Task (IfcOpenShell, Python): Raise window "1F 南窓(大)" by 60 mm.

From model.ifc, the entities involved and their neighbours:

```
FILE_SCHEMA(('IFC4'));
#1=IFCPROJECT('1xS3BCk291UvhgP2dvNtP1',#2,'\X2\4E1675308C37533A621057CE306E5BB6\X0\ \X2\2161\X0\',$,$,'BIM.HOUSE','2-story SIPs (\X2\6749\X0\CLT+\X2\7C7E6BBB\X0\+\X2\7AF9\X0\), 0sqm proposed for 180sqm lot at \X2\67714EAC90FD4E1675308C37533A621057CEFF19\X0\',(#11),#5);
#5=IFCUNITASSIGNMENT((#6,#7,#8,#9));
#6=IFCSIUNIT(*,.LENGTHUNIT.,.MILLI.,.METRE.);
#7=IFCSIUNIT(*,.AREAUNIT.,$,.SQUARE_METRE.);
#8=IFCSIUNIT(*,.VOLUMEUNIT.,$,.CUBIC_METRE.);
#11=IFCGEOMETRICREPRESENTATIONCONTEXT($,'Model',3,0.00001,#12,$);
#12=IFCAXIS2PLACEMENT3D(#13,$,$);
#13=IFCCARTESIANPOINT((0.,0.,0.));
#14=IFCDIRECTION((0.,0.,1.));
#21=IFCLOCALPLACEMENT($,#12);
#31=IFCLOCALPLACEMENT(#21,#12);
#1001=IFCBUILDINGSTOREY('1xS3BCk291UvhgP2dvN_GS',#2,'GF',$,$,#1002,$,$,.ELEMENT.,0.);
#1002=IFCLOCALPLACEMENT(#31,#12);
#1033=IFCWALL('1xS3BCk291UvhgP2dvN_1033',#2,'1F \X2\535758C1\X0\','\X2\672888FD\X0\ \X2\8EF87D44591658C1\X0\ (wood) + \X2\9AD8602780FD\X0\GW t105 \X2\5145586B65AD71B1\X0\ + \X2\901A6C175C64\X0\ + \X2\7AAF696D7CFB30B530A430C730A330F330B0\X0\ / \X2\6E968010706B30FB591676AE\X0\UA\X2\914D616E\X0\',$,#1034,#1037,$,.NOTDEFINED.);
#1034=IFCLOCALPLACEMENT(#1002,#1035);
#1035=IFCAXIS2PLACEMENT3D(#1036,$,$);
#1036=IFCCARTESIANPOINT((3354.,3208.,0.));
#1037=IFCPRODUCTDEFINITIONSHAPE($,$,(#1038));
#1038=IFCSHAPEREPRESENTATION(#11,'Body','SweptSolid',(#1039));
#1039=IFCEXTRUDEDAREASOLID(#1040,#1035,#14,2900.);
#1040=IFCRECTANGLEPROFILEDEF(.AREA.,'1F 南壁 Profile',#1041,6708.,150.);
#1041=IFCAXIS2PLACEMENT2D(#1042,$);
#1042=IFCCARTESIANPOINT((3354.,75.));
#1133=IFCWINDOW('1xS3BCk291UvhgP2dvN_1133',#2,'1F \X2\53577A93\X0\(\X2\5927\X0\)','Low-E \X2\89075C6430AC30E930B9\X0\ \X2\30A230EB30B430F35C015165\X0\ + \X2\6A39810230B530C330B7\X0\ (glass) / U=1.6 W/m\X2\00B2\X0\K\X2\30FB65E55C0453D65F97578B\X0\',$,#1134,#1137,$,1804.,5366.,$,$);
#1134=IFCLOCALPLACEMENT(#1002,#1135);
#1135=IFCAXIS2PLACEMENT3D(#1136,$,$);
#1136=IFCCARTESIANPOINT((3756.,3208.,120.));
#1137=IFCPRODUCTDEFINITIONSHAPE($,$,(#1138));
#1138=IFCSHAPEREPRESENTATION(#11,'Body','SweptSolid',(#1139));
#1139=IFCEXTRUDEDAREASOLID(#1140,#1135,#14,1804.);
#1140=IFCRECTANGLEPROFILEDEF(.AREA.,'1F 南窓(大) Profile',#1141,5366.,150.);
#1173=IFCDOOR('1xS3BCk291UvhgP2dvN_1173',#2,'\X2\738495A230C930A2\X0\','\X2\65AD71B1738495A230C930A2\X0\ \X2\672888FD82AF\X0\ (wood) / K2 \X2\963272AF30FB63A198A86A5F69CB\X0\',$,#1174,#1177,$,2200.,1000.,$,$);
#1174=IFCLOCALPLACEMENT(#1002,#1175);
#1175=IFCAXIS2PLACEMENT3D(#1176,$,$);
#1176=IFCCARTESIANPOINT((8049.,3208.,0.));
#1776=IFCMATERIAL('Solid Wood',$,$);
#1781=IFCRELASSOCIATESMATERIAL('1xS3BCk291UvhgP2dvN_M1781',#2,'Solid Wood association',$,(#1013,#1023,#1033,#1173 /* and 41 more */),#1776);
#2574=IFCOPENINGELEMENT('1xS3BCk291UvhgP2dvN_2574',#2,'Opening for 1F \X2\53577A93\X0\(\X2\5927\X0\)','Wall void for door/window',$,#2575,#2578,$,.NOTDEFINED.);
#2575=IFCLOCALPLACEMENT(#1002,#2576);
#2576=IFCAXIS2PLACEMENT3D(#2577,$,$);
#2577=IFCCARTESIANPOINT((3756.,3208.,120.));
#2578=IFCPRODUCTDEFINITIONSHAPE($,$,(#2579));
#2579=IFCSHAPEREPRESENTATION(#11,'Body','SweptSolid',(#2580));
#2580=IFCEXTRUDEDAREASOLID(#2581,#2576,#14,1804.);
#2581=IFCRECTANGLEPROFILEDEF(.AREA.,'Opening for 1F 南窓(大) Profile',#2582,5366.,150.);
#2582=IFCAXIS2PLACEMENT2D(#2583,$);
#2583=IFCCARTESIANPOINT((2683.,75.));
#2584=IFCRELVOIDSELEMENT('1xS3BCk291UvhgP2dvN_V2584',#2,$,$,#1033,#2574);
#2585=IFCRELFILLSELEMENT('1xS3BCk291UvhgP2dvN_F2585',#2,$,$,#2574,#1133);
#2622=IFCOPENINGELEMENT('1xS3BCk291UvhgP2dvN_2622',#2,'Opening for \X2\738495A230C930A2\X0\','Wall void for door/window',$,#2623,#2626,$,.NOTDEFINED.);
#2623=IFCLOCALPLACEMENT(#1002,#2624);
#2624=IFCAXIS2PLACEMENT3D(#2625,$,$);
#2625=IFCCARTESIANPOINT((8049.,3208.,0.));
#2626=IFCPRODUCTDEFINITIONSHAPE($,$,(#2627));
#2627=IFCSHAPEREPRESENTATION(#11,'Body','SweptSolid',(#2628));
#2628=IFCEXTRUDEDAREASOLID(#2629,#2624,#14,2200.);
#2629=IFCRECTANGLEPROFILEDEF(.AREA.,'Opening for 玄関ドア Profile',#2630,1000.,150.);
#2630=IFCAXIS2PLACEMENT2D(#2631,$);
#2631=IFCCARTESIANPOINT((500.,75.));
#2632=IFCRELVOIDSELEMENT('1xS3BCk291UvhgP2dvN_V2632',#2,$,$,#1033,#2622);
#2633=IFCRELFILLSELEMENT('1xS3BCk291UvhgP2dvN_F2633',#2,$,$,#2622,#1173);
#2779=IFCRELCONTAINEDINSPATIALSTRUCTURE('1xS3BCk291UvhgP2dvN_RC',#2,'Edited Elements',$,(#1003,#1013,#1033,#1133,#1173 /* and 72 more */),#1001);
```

```python
import numpy as np
import ifcopenshell
import ifcopenshell.api.geometry
import ifcopenshell.util.placement
import ifcopenshell.util.unit

model = ifcopenshell.open("model.ifc")
unit_scale = ifcopenshell.util.unit.calculate_unit_scale(model)

window = model.by_guid("1xS3BCk291UvhgP2dvN_1133")
opening = window.FillsVoids[0].RelatingOpeningElement
dz = 60.0

shift = np.array([0.0, 0.0, dz])
# The window is not placed relative to its opening, so move both.
for product in (opening, window):
    matrix = ifcopenshell.util.placement.get_local_placement(product.ObjectPlacement)
    matrix[:3, 3] += shift
    ifcopenshell.api.geometry.edit_object_placement(model, product=product, matrix=matrix, is_si=False)

print(f"moved by {dz * unit_scale:+.3f} m")

model.write("model_edited.ifc")
```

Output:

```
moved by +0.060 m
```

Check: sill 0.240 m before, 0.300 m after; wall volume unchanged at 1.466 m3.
